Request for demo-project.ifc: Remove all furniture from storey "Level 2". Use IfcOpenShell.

First a look at what the model holds.

```python
import ifcopenshell
import ifcopenshell.util.element

model = ifcopenshell.open("demo-project.ifc")
print(model.schema)
storey = next(s for s in model.by_type("IfcBuildingStorey") if s.Name == "Level 2")
furniture = [e for e in ifcopenshell.util.element.get_decomposition(storey) if e.is_a("IfcFurnishingElement")]
seen = {}
for e in furniture:
    element_type = ifcopenshell.util.element.get_type(e)
    name = element_type.Name if element_type not in (None, e) else None
    seen[name] = seen.get(name, 0) + 1
for name, count in sorted(seen.items(), key=str):
    print(count, "x", name)
```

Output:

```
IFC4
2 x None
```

```python
import ifcopenshell
import ifcopenshell.api.root
import ifcopenshell.util.element

model = ifcopenshell.open("demo-project.ifc")

storey = next(s for s in model.by_type("IfcBuildingStorey") if s.Name == "Level 2")
furniture = [e for e in ifcopenshell.util.element.get_decomposition(storey) if e.is_a("IfcFurnishingElement")]

for e in furniture:
    ifcopenshell.api.root.remove_product(model, product=e)
print(len(furniture), "removed")

model.write("demo-project_edited.ifc")
```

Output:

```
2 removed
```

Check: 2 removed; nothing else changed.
